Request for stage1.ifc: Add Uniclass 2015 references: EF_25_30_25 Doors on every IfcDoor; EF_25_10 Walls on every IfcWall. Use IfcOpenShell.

First a look at what the model holds.

```python
import ifcopenshell

model = ifcopenshell.open("stage1.ifc")
print(model.schema)
print("classifications:", [c.Name for c in model.by_type("IfcClassification")])
for ifc_class in ("IfcDoor", "IfcRoof", "IfcStair", "IfcWall", "IfcWindow"):
    print(ifc_class, len(model.by_type(ifc_class)))
```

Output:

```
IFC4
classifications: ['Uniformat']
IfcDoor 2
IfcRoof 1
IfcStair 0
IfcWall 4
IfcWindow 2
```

```python
import ifcopenshell
import ifcopenshell.api.classification

model = ifcopenshell.open("stage1.ifc")

system = ifcopenshell.api.classification.add_classification(model, classification="Uniclass 2015")

codes = {
    "IfcDoor": ("EF_25_30_25", "Doors"),
    "IfcWall": ("EF_25_10", "Walls"),
}
for ifc_class, (code, name) in codes.items():
    products = model.by_type(ifc_class)
    ifcopenshell.api.classification.add_reference(
        model, products=products, classification=system, identification=code, name=name
    )
    print(code, len(products))

model.write("stage1-out.ifc")
```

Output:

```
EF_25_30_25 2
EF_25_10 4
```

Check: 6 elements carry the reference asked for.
